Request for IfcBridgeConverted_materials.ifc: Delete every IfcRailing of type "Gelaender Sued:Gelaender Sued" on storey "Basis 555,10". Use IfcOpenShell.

First a look at what the model holds.

```python
import ifcopenshell
import ifcopenshell.util.element

model = ifcopenshell.open("IfcBridgeConverted_materials.ifc")
print(model.schema)
storey = next(s for s in model.by_type("IfcBuildingStorey") if s.Name == "Basis 555,10")
railings = [e for e in ifcopenshell.util.element.get_decomposition(storey) if e.is_a("IfcRailing")]
seen = {}
for e in railings:
    element_type = ifcopenshell.util.element.get_type(e)
    name = element_type.Name if element_type not in (None, e) else None
    seen[name] = seen.get(name, 0) + 1
for name, count in sorted(seen.items(), key=str):
    print(count, "x", name)
```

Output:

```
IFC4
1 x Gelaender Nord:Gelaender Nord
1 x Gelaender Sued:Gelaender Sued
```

```python
import ifcopenshell
import ifcopenshell.api.root
import ifcopenshell.util.element

model = ifcopenshell.open("IfcBridgeConverted_materials.ifc")

storey = next(s for s in model.by_type("IfcBuildingStorey") if s.Name == "Basis 555,10")
railings = [e for e in ifcopenshell.util.element.get_decomposition(storey) if e.is_a("IfcRailing")]
targets = [e for e in railings if (t := ifcopenshell.util.element.get_type(e)) not in (None, e) and t.Name == "Gelaender Sued:Gelaender Sued"]

for e in targets:
    ifcopenshell.api.root.remove_product(model, product=e)
print(len(targets), "removed")

model.write("IfcBridgeConverted_materials_updated.ifc")
```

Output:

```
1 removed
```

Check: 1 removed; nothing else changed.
